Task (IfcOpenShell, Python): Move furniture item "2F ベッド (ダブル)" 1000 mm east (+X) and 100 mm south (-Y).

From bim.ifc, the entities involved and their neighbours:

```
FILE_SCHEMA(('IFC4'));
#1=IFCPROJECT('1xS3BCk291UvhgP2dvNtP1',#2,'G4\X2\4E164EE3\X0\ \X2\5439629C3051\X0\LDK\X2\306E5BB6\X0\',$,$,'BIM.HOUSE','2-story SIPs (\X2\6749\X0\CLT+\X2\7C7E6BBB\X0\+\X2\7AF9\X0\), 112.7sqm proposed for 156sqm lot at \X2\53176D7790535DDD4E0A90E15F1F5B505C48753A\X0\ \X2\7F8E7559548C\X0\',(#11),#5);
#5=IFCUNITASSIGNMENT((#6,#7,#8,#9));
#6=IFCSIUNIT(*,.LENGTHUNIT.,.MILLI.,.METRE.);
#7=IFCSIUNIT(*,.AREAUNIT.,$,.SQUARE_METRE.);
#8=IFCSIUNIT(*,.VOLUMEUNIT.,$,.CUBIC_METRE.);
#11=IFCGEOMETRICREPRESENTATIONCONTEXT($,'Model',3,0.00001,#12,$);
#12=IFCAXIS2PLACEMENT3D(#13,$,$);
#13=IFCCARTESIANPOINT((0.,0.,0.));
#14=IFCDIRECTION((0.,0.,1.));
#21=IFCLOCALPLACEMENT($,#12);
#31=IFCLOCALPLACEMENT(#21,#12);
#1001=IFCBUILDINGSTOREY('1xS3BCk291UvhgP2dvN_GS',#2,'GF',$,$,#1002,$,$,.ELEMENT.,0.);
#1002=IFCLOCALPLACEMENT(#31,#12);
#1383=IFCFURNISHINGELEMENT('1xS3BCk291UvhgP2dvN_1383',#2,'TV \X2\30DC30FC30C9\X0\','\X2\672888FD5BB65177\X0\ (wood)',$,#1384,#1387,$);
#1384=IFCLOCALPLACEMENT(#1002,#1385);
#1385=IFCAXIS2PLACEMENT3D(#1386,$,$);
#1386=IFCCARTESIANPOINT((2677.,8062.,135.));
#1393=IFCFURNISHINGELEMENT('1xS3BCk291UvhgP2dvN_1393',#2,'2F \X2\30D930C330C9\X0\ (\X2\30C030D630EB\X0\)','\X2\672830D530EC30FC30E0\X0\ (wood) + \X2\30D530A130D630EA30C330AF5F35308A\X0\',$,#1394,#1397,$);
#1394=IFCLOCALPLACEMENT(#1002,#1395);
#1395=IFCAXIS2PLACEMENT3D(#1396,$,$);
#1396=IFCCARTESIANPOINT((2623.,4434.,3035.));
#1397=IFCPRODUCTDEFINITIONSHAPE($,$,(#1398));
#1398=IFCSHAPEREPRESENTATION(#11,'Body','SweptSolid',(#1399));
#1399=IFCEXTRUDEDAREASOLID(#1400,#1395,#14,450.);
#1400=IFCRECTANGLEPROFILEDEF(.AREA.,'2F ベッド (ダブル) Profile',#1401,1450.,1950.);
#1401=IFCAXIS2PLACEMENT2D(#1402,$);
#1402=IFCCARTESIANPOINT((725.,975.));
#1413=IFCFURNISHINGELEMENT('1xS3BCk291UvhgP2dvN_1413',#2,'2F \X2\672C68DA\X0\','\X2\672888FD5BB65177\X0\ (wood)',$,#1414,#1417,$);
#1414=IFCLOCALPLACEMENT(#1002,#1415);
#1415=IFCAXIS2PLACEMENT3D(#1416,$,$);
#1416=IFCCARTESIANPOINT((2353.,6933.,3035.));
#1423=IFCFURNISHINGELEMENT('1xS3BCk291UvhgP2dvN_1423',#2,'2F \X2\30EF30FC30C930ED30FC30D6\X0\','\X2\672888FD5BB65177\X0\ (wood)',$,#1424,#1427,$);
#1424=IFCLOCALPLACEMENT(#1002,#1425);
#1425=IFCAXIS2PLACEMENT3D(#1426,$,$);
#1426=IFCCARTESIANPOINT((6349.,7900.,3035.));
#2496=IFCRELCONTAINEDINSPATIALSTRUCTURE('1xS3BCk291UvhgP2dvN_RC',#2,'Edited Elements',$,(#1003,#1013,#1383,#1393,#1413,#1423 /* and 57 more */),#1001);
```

```python
import ifcopenshell
import ifcopenshell.api.geometry
import ifcopenshell.util.placement

model = ifcopenshell.open("bim.ifc")

item = model.by_id(1393)
matrix = ifcopenshell.util.placement.get_local_placement(item.ObjectPlacement)
matrix[0, 3] += 1000.0
matrix[1, 3] -= 100.0
ifcopenshell.api.geometry.edit_object_placement(model, product=item, matrix=matrix, is_si=False)

print(ifcopenshell.util.placement.get_local_placement(item.ObjectPlacement).round(3) + 0.0)

model.write("bim_rev.ifc")
```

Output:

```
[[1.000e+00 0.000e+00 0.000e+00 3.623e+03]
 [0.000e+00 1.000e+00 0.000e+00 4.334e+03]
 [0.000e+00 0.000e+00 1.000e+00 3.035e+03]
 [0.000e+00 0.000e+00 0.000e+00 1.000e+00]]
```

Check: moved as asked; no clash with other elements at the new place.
